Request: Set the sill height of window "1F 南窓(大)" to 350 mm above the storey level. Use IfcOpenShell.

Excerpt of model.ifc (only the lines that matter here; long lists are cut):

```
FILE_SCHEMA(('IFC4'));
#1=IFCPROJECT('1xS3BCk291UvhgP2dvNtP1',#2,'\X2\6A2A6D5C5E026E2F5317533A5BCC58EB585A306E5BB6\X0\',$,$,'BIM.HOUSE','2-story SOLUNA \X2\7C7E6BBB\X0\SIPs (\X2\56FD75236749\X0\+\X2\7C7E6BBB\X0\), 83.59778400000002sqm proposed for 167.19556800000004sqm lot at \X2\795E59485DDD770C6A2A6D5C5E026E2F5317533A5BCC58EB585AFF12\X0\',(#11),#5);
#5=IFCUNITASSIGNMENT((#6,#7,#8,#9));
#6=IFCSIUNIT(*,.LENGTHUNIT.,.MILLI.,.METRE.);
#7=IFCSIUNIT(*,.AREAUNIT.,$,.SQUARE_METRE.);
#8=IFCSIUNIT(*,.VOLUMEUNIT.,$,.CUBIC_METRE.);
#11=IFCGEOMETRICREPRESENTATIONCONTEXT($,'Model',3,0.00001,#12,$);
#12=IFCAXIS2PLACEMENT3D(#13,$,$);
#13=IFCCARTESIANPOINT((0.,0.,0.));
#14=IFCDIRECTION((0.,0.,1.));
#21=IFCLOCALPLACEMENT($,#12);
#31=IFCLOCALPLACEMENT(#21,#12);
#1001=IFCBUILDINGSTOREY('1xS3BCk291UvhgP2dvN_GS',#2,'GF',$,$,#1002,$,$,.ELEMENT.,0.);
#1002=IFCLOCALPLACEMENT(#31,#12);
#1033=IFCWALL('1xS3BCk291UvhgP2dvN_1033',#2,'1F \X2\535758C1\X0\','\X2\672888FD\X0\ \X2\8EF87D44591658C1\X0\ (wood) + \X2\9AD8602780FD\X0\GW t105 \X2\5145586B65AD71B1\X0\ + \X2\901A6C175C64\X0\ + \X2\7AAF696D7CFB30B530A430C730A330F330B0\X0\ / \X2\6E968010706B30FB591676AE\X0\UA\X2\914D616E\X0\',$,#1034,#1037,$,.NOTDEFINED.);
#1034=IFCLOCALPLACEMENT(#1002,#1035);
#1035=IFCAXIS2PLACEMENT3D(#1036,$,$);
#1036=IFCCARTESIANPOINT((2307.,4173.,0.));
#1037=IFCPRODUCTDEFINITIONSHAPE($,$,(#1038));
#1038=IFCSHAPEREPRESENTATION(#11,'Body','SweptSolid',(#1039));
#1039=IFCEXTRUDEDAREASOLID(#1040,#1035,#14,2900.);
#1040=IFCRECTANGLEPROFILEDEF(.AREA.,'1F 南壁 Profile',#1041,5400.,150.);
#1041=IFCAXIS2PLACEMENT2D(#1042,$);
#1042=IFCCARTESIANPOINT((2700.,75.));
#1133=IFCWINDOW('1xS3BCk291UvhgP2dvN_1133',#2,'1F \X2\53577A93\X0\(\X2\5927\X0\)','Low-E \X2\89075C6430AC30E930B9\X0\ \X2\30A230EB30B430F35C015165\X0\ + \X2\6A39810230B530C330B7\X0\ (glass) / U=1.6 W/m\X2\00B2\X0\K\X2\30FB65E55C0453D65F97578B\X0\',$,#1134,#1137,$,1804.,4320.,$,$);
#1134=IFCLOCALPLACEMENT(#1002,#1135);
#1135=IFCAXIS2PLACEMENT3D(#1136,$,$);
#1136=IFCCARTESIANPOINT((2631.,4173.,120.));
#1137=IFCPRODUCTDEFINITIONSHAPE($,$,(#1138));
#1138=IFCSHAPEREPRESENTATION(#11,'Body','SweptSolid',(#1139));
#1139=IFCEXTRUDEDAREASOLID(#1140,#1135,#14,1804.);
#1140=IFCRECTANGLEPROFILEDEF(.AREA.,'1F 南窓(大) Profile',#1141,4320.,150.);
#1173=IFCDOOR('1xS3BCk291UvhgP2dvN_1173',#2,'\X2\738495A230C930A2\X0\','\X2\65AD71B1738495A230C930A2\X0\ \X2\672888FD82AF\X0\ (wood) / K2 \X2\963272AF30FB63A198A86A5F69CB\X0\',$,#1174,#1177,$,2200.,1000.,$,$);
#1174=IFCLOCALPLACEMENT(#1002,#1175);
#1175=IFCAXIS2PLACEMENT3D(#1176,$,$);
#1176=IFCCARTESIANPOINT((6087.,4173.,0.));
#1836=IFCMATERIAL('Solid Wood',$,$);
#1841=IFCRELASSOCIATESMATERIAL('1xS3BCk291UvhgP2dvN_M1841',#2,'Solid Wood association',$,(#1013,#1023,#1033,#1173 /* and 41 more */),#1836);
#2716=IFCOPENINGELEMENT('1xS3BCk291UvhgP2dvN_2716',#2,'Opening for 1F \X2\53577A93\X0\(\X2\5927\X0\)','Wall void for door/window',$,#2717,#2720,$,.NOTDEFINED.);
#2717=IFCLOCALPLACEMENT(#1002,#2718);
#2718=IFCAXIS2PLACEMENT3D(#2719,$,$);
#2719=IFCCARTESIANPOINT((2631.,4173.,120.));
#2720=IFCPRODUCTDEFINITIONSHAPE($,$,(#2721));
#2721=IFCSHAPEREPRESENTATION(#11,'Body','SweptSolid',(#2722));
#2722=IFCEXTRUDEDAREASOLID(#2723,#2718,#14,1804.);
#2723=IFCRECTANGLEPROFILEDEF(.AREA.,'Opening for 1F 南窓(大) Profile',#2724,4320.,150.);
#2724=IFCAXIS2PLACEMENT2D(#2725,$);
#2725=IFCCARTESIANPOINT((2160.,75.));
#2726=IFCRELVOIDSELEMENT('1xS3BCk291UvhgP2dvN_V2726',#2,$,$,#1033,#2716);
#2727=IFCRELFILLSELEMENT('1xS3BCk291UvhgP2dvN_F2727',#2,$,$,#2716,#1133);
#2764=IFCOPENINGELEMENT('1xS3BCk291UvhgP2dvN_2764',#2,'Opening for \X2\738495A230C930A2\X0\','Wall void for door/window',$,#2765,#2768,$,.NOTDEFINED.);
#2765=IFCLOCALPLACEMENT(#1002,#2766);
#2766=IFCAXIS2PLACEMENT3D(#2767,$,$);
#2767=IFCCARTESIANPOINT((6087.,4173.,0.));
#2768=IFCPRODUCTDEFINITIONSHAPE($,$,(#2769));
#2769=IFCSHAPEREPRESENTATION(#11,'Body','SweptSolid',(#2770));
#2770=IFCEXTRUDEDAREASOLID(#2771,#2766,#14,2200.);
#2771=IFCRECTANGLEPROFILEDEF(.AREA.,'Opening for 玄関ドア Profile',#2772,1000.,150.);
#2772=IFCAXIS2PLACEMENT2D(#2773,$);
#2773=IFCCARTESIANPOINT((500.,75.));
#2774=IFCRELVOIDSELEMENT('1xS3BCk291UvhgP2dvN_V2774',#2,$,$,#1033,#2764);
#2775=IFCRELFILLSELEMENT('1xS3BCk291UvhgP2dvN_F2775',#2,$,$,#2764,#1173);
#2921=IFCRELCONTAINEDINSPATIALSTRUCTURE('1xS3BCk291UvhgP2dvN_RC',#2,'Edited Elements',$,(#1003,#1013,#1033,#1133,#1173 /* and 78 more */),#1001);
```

```python
import numpy as np
import ifcopenshell
import ifcopenshell.api.geometry
import ifcopenshell.geom
import ifcopenshell.util.element
import ifcopenshell.util.placement
import ifcopenshell.util.shape
import ifcopenshell.util.unit

model = ifcopenshell.open("model.ifc")
unit_scale = ifcopenshell.util.unit.calculate_unit_scale(model)

window = model.by_guid("1xS3BCk291UvhgP2dvN_1133")
opening = window.FillsVoids[0].RelatingOpeningElement
storey = ifcopenshell.util.element.get_container(window, ifc_class="IfcBuildingStorey")
level = ifcopenshell.util.placement.get_local_placement(storey.ObjectPlacement)[2, 3]

# The opening's origin need not be at the sill, so measure its lowest point.
shape = ifcopenshell.geom.create_shape(ifcopenshell.geom.settings(), opening)
bottom = ifcopenshell.util.shape.get_shape_bottom_elevation(shape, shape.geometry) / unit_scale
dz = level + 0.35 / unit_scale - bottom

shift = np.array([0.0, 0.0, dz])
# The window is not placed relative to its opening, so move both.
for product in (opening, window):
    matrix = ifcopenshell.util.placement.get_local_placement(product.ObjectPlacement)
    matrix[:3, 3] += shift
    ifcopenshell.api.geometry.edit_object_placement(model, product=product, matrix=matrix, is_si=False)

print(f"moved by {dz * unit_scale:+.3f} m")

model.write("model-out.ifc")
```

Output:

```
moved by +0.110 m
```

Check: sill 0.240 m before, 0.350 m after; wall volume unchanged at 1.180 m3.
